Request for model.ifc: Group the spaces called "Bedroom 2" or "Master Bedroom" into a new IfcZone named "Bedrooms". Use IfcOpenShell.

First a look at what the model holds.

```python
import ifcopenshell

model = ifcopenshell.open("model.ifc")
print(model.schema)
seen = {}
for space in model.by_type("IfcSpace"):
    seen[space.LongName] = seen.get(space.LongName, 0) + 1
for name, count in sorted(seen.items(), key=str):
    print(count, "x", name)
print("zones:", [z.Name for z in model.by_type("IfcZone")][:20])
```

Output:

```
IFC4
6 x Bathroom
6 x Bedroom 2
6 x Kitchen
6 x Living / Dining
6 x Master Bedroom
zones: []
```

```python
import ifcopenshell
import ifcopenshell.api.group
import ifcopenshell.api.root

model = ifcopenshell.open("model.ifc")

names = {"Bedroom 2", "Master Bedroom"}
spaces = [s for s in model.by_type("IfcSpace") if s.LongName in names]

zone = ifcopenshell.api.root.create_entity(model, ifc_class="IfcZone", name="Bedrooms")
ifcopenshell.api.group.assign_group(model, products=spaces, group=zone)
print(len(spaces), "spaces in", zone.Name)

model.write("model_rev.ifc")
```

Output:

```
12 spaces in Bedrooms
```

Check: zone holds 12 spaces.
